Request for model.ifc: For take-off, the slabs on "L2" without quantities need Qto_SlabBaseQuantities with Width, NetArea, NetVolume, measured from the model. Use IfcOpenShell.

First a look at what the model holds.

```python
import ifcopenshell
import ifcopenshell.util.element
import ifcopenshell.util.unit

model = ifcopenshell.open("model.ifc")
print(model.schema)
for unit_type in ("LENGTHUNIT", "AREAUNIT", "VOLUMEUNIT"):
    print(unit_type, ifcopenshell.util.unit.calculate_unit_scale(model, unit_type))
storey = next(s for s in model.by_type("IfcBuildingStorey") if s.Name == "L2")
slabs = [e for e in ifcopenshell.util.element.get_decomposition(storey) if e.is_a("IfcSlab")]
for e in sorted(slabs, key=lambda e: e.id()):
    print(e.id(), e.is_a(), e.Name, list(ifcopenshell.util.element.get_psets(e, qtos_only=True)), sep=" | ")
```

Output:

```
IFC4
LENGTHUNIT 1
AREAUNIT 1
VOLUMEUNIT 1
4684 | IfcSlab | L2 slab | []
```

```python
import ifcopenshell
import ifcopenshell.api.pset
import ifcopenshell.geom
import ifcopenshell.util.element
import ifcopenshell.util.shape
import ifcopenshell.util.unit

model = ifcopenshell.open("model.ifc")
unit_scale = ifcopenshell.util.unit.calculate_unit_scale(model)
area_scale = ifcopenshell.util.unit.calculate_unit_scale(model, "AREAUNIT")
volume_scale = ifcopenshell.util.unit.calculate_unit_scale(model, "VOLUMEUNIT")
settings = ifcopenshell.geom.settings()

storey = next(s for s in model.by_type("IfcBuildingStorey") if s.Name == "L2")
slabs = [e for e in ifcopenshell.util.element.get_decomposition(storey) if e.is_a("IfcSlab")]

for e in sorted(slabs, key=lambda e: e.id()):
    if ifcopenshell.util.element.get_psets(e, qtos_only=True, should_inherit=False):
        continue
    # Geometry comes back in metres, in the element's own axes.
    shape = ifcopenshell.geom.create_shape(settings, e)
    values = {
        "Width": ifcopenshell.util.shape.get_z(shape.geometry) / unit_scale,
        "NetArea": ifcopenshell.util.shape.get_footprint_area(shape.geometry) / area_scale,
        "NetVolume": ifcopenshell.util.shape.get_volume(shape.geometry) / volume_scale,
    }
    qto = ifcopenshell.api.pset.add_qto(model, product=e, name="Qto_SlabBaseQuantities")
    ifcopenshell.api.pset.edit_qto(model, qto=qto, properties=values)
    print(e.id(), {k: round(v, 3) for k, v in values.items()})

model.write("model_v2.ifc")
```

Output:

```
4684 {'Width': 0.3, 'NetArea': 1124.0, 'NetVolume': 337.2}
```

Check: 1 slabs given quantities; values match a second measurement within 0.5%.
